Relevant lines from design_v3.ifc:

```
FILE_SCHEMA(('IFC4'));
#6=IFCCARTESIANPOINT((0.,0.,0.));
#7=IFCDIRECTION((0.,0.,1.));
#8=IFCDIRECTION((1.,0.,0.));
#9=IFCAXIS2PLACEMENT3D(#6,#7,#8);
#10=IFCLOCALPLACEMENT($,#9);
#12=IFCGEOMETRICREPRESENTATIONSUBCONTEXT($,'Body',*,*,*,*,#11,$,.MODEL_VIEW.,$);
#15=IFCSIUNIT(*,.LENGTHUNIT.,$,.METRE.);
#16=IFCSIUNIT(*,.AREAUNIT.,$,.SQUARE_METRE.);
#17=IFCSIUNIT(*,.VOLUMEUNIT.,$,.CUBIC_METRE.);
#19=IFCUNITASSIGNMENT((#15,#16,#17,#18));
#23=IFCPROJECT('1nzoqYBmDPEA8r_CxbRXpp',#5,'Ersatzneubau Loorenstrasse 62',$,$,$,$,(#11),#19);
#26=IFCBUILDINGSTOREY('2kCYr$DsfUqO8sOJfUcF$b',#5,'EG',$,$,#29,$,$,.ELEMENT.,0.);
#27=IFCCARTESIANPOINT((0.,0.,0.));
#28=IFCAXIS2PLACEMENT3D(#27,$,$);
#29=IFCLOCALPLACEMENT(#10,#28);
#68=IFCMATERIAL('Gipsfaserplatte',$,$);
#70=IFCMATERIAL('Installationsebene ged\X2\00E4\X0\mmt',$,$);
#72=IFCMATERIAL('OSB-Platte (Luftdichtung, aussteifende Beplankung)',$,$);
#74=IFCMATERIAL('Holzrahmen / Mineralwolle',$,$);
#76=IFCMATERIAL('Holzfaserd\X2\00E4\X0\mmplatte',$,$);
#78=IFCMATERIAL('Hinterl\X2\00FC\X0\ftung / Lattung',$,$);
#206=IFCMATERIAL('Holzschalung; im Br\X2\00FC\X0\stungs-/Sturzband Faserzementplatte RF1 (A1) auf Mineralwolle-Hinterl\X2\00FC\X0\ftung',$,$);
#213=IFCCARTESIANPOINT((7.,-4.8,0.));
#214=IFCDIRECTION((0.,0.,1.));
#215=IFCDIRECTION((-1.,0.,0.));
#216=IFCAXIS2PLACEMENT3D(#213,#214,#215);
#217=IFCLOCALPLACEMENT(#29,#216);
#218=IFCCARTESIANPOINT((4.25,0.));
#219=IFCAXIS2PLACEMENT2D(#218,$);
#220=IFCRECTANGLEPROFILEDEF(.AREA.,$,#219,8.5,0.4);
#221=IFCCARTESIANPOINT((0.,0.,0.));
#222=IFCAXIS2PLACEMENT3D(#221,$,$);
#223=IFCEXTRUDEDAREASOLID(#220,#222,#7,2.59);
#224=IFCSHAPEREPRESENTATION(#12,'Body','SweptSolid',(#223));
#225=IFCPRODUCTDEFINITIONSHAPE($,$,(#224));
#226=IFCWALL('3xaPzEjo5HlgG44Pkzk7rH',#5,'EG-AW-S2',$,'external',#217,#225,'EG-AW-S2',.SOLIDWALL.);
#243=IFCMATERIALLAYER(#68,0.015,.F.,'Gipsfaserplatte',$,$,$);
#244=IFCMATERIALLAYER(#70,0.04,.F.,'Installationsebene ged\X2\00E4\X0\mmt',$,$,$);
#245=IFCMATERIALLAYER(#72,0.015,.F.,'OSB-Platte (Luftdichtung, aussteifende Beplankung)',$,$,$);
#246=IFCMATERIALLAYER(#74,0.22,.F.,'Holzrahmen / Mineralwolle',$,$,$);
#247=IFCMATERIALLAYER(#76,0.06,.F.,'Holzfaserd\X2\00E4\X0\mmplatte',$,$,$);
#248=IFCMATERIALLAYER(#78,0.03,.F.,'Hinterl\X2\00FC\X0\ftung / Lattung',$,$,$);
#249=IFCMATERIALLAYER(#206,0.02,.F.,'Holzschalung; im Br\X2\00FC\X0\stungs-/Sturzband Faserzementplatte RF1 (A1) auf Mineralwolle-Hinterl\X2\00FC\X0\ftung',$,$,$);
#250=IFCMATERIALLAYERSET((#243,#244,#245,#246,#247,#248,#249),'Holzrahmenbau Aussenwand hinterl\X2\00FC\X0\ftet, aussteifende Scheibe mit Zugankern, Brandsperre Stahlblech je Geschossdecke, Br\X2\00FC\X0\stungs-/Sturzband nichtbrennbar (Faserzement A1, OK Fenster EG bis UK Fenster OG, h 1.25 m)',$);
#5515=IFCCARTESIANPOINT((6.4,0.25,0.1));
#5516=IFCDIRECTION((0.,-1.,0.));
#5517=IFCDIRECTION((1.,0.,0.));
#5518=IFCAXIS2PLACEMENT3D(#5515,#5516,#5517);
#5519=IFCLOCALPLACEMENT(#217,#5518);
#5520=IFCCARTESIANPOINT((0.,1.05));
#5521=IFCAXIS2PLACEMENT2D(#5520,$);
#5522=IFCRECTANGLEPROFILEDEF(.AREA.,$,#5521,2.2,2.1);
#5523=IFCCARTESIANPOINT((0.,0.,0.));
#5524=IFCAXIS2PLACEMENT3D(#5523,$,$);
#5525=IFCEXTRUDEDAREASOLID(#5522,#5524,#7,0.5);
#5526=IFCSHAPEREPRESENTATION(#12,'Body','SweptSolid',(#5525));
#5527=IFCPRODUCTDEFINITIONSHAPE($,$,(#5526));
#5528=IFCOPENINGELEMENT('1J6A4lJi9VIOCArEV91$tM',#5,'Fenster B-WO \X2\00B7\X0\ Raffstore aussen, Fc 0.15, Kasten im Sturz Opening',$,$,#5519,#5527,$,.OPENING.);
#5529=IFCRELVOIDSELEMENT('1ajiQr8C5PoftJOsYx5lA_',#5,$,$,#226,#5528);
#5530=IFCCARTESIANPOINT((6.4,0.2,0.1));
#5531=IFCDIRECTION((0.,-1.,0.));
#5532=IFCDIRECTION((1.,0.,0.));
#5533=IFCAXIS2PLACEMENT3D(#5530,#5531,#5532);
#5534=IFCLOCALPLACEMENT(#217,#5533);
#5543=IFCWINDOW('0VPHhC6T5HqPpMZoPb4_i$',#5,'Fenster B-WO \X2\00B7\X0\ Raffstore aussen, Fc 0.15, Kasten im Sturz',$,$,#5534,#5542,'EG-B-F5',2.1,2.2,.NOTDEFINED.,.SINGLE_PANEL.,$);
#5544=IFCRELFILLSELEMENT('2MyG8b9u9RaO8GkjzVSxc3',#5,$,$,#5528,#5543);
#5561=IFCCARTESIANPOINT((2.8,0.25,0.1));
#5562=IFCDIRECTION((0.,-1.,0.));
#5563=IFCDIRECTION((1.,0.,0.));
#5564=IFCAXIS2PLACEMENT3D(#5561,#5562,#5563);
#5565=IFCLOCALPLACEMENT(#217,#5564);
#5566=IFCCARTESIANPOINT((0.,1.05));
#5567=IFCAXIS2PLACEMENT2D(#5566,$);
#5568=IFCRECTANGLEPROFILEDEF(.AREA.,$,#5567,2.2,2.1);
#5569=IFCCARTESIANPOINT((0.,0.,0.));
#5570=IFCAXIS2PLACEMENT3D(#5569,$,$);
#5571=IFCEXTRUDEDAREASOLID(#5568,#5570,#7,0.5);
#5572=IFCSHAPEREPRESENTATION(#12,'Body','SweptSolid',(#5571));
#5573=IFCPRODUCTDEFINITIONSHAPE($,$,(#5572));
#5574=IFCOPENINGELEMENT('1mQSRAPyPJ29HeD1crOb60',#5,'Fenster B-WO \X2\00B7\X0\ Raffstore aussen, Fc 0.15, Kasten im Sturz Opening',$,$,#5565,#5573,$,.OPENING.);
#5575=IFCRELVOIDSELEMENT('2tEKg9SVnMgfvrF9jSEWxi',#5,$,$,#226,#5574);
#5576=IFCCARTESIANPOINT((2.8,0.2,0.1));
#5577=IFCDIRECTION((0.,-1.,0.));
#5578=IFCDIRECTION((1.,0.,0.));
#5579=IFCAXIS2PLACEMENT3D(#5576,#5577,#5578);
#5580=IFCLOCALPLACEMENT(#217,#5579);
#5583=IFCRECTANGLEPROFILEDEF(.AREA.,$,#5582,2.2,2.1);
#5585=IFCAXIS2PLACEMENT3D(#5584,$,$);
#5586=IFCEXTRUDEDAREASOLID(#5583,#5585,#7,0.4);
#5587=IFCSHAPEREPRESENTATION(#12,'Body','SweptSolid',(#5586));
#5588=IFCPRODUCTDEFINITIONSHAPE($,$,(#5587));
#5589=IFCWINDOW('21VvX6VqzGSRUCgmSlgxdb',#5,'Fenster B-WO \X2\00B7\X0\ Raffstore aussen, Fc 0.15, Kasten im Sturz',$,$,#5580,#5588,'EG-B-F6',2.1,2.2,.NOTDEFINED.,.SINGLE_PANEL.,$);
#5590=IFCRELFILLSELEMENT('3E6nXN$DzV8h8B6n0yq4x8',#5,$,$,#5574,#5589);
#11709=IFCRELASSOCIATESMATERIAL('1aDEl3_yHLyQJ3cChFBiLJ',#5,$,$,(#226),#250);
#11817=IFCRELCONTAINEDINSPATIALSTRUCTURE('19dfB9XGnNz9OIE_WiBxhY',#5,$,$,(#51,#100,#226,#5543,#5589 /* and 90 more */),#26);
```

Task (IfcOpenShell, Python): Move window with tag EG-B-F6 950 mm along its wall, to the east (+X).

```python
import ifcopenshell
import ifcopenshell.api.geometry
import ifcopenshell.util.placement
import ifcopenshell.util.unit

model = ifcopenshell.open("design_v3.ifc")
unit_scale = ifcopenshell.util.unit.calculate_unit_scale(model)

window = model.by_guid("21VvX6VqzGSRUCgmSlgxdb")
opening = window.FillsVoids[0].RelatingOpeningElement
wall = opening.VoidsElements[0].RelatingBuildingElement

wall_matrix = ifcopenshell.util.placement.get_local_placement(wall.ObjectPlacement)
shift = wall_matrix[:3, 0] * -0.95 / unit_scale
before = ifcopenshell.util.placement.get_local_placement(window.ObjectPlacement)[:3, 3].copy()

# The window is not placed relative to its opening, so move both.
for product in (opening, window):
    matrix = ifcopenshell.util.placement.get_local_placement(product.ObjectPlacement)
    matrix[:3, 3] += shift
    ifcopenshell.api.geometry.edit_object_placement(model, product=product, matrix=matrix, is_si=False)

after = ifcopenshell.util.placement.get_local_placement(window.ObjectPlacement)[:3, 3]
print("window moved by", (after - before).round(3) + 0.0)

model.write("design_v3_edited.ifc")
```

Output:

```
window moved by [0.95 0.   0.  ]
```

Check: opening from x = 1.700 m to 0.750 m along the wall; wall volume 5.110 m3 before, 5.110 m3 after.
